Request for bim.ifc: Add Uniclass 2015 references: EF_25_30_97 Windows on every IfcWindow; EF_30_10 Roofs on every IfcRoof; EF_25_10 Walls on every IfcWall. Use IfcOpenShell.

First a look at what the model holds.

```python
import ifcopenshell

model = ifcopenshell.open("bim.ifc")
print(model.schema)
print("classifications:", [c.Name for c in model.by_type("IfcClassification")])
for ifc_class in ("IfcDoor", "IfcRoof", "IfcStair", "IfcWall", "IfcWindow"):
    print(ifc_class, len(model.by_type(ifc_class)))
```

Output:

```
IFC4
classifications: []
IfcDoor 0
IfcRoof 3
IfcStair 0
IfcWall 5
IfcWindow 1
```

```python
import ifcopenshell
import ifcopenshell.api.classification

model = ifcopenshell.open("bim.ifc")

system = ifcopenshell.api.classification.add_classification(model, classification="Uniclass 2015")

codes = {
    "IfcWindow": ("EF_25_30_97", "Windows"),
    "IfcRoof": ("EF_30_10", "Roofs"),
    "IfcWall": ("EF_25_10", "Walls"),
}
for ifc_class, (code, name) in codes.items():
    products = model.by_type(ifc_class)
    ifcopenshell.api.classification.add_reference(
        model, products=products, classification=system, identification=code, name=name
    )
    print(code, len(products))

model.write("bim_edited.ifc")
```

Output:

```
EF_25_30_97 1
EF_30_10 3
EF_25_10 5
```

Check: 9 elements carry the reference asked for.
